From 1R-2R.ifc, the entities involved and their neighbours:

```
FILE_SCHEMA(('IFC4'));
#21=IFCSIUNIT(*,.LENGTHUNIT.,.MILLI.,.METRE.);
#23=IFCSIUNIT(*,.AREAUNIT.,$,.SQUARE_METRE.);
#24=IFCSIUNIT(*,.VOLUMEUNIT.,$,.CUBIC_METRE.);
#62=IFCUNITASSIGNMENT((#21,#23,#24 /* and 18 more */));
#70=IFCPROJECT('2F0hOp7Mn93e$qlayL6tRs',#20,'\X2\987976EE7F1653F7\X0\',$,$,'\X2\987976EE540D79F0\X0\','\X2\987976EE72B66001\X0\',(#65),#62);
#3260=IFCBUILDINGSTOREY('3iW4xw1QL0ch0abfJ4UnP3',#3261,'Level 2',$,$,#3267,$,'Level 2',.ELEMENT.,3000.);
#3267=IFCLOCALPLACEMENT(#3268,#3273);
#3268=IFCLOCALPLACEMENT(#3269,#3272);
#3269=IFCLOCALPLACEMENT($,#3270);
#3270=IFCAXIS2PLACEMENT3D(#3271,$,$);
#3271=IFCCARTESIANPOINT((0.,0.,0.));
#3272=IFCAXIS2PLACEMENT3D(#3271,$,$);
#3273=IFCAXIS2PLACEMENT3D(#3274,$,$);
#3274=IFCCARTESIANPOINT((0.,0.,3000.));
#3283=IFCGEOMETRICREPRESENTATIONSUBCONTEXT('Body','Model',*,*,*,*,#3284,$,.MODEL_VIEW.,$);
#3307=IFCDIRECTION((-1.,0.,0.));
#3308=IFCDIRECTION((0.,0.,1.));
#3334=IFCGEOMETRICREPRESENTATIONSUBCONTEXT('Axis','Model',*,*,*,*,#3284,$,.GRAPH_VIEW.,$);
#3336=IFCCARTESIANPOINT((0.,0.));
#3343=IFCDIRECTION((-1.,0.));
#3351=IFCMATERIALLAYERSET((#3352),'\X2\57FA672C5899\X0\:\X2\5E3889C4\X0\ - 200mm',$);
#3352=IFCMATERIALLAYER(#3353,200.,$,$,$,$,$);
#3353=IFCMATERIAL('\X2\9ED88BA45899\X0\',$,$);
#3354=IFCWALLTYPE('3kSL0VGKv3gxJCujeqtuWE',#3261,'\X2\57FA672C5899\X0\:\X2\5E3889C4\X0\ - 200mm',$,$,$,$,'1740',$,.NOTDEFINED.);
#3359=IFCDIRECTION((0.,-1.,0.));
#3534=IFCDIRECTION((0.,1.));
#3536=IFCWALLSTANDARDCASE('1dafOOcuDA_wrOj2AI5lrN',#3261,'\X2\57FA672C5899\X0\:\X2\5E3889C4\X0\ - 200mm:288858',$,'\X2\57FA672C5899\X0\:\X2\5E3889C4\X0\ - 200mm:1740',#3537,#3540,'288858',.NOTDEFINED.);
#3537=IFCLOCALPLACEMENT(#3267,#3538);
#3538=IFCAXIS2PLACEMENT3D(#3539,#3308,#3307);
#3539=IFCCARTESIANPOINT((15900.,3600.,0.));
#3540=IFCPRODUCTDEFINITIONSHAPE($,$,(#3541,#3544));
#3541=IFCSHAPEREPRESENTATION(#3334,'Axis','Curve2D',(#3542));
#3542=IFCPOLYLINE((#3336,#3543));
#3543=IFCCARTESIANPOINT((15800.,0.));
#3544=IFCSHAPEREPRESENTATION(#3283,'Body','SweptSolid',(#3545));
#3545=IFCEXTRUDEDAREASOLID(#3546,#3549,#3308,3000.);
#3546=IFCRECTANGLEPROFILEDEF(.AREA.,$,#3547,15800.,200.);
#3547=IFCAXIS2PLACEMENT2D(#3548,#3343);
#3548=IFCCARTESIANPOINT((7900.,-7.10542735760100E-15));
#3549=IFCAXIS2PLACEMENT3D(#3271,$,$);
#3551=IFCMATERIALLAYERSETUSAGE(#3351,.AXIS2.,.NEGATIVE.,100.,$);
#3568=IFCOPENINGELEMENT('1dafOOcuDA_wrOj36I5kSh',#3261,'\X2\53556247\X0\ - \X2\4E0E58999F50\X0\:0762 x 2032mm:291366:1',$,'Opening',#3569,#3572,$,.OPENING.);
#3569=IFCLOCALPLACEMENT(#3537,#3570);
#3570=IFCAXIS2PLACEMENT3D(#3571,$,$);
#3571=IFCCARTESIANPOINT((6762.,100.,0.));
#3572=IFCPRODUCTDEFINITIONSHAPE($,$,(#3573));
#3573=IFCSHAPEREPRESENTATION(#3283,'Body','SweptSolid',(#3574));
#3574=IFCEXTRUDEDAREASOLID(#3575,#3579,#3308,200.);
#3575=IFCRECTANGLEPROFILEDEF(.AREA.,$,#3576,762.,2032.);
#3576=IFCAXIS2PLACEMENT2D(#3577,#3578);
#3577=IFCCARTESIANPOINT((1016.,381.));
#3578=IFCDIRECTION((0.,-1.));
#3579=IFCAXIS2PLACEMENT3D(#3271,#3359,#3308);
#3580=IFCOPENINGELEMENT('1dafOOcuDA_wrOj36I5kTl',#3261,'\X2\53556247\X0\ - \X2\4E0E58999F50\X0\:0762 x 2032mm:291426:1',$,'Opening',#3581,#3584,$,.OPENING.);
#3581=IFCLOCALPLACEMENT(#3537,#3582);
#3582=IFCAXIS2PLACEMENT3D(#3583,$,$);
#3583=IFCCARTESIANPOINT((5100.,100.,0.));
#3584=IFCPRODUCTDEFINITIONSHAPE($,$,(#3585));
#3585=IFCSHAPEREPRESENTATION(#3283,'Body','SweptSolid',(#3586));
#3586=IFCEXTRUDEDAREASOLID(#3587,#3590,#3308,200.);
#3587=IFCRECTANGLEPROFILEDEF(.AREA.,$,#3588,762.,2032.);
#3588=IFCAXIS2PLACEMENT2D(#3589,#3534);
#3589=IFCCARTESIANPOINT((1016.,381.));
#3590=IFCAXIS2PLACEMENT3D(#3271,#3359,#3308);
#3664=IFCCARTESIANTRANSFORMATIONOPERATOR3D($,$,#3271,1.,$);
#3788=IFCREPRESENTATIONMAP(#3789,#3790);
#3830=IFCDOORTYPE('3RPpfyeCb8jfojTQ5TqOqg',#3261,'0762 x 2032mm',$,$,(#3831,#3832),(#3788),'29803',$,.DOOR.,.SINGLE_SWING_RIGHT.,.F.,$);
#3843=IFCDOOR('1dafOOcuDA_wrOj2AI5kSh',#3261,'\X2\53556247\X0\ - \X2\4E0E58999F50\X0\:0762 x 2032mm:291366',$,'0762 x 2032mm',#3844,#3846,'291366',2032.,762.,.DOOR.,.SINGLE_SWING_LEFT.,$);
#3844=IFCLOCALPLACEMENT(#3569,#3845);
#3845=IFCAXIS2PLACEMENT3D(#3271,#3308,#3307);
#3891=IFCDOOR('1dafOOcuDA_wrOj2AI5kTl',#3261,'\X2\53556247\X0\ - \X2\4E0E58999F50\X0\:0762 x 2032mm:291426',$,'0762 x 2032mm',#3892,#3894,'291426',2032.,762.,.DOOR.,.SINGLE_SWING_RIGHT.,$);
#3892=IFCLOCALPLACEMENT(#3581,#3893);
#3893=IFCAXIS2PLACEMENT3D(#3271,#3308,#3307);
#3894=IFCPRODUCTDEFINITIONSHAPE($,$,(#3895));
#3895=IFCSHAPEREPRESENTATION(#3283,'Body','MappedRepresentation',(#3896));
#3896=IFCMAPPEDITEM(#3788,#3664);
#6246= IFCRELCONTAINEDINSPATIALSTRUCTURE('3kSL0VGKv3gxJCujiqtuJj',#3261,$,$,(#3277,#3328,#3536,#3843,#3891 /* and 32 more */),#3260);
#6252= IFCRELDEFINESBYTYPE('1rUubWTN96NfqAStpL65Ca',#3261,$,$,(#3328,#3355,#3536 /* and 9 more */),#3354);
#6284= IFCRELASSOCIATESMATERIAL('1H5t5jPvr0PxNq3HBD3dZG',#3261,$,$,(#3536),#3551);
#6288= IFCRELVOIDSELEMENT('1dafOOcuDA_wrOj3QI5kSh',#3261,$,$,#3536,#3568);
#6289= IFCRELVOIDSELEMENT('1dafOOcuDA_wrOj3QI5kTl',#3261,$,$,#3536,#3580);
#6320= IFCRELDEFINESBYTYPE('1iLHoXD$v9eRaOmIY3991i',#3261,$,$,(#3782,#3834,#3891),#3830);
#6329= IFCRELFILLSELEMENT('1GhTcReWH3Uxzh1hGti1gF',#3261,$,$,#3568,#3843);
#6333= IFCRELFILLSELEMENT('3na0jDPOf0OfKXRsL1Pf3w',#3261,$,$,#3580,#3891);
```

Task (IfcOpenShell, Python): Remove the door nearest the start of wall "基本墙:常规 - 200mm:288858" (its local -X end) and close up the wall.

```python
import ifcopenshell
import ifcopenshell.api.feature
import ifcopenshell.api.root
import ifcopenshell.geom
import ifcopenshell.util.shape

model = ifcopenshell.open("1R-2R.ifc")
settings = ifcopenshell.geom.settings()


def volume(element):
    """Net volume in cubic metres, openings subtracted."""
    shape = ifcopenshell.geom.create_shape(settings, element)
    return ifcopenshell.util.shape.get_volume(shape.geometry)


door = model.by_guid("1dafOOcuDA_wrOj2AI5kTl")
opening = door.FillsVoids[0].RelatingOpeningElement
wall = opening.VoidsElements[0].RelatingBuildingElement
before = volume(wall)

ifcopenshell.api.root.remove_product(model, product=door)
ifcopenshell.api.feature.remove_feature(model, feature=opening)

after = volume(wall)

print(f"wall volume {before:.3f} -> {after:.3f} m3")

model.write("1R-2R_v2.ifc")
```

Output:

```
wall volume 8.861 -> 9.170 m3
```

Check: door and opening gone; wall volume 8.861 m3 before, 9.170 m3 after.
